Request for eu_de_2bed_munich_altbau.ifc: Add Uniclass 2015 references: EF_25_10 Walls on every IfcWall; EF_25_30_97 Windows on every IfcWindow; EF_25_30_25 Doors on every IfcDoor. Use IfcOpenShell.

First a look at what the model holds.

```python
import ifcopenshell

model = ifcopenshell.open("eu_de_2bed_munich_altbau.ifc")
print(model.schema)
print("classifications:", [c.Name for c in model.by_type("IfcClassification")])
for ifc_class in ("IfcDoor", "IfcRoof", "IfcStair", "IfcWall", "IfcWindow"):
    print(ifc_class, len(model.by_type(ifc_class)))
```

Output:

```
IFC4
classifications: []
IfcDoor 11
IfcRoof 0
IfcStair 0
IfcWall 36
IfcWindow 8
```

```python
import ifcopenshell
import ifcopenshell.api.classification

model = ifcopenshell.open("eu_de_2bed_munich_altbau.ifc")

system = ifcopenshell.api.classification.add_classification(model, classification="Uniclass 2015")

codes = {
    "IfcWall": ("EF_25_10", "Walls"),
    "IfcWindow": ("EF_25_30_97", "Windows"),
    "IfcDoor": ("EF_25_30_25", "Doors"),
}
for ifc_class, (code, name) in codes.items():
    products = model.by_type(ifc_class)
    ifcopenshell.api.classification.add_reference(
        model, products=products, classification=system, identification=code, name=name
    )
    print(code, len(products))

model.write("eu_de_2bed_munich_altbau_edited.ifc")
```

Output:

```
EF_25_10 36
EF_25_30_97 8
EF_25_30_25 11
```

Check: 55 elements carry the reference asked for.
